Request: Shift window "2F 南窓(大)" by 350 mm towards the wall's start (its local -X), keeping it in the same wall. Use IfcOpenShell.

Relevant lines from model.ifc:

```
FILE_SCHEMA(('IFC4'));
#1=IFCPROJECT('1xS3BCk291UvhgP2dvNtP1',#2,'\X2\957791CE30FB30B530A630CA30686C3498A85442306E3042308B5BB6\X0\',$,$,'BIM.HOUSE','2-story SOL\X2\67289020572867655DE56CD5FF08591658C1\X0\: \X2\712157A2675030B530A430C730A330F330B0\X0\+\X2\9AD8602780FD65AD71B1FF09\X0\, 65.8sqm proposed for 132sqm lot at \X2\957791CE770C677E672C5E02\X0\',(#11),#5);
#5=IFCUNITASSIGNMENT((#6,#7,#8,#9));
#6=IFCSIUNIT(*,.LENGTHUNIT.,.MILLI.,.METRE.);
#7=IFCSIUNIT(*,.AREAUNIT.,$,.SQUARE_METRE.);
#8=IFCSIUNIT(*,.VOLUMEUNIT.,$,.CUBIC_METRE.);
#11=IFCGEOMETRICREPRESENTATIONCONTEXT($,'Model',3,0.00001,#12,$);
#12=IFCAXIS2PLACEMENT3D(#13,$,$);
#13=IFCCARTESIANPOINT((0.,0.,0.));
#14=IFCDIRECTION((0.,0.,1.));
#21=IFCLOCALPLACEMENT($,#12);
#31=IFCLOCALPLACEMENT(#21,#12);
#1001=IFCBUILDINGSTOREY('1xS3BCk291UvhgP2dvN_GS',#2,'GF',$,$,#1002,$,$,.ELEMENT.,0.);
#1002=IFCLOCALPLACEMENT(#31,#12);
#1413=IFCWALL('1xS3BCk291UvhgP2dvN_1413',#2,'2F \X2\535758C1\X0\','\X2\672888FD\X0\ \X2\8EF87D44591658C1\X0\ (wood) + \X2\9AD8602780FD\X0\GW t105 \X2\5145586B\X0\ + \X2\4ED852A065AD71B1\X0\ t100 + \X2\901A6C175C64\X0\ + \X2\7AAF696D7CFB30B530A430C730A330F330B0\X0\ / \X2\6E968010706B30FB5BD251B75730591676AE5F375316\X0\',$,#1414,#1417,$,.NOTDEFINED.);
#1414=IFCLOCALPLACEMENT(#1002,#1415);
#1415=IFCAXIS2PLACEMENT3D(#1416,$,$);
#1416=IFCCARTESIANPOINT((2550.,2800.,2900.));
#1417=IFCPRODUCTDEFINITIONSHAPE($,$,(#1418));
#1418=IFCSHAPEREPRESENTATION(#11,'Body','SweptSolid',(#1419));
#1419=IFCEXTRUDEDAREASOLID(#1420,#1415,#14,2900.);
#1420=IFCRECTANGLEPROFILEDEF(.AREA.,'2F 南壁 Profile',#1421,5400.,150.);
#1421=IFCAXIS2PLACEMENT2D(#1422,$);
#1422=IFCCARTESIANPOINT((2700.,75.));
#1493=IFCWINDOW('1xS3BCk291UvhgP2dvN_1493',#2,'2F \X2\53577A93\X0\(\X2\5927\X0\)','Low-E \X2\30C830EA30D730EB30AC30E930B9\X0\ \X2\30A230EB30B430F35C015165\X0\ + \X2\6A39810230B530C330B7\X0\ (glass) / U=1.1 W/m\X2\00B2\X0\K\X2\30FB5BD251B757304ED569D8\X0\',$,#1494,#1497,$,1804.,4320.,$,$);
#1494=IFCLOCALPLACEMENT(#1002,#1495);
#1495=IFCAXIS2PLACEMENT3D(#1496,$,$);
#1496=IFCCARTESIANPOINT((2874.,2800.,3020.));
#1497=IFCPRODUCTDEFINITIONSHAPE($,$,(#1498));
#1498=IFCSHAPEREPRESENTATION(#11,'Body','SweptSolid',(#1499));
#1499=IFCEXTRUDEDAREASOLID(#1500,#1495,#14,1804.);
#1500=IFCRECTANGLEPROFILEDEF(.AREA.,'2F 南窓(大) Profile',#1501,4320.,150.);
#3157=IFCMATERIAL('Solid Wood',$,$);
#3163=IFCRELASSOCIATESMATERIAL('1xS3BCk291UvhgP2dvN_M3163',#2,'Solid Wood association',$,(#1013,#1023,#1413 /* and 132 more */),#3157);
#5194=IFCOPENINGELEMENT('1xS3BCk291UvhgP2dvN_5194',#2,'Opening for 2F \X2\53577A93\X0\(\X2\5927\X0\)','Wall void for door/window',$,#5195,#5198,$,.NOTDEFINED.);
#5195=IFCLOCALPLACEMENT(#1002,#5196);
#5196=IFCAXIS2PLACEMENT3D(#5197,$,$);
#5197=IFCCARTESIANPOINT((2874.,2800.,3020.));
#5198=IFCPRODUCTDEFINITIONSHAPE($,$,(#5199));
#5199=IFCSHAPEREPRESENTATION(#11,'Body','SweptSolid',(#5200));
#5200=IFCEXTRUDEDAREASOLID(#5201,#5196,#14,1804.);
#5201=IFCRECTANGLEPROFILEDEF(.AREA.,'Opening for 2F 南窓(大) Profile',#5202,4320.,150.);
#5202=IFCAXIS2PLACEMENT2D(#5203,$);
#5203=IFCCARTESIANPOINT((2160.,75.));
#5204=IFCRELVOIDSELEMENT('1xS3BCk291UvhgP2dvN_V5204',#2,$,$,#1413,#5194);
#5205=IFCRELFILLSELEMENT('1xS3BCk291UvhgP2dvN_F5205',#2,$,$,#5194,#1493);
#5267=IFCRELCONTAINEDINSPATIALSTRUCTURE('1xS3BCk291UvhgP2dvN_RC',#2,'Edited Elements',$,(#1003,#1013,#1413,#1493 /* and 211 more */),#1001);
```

```python
import ifcopenshell
import ifcopenshell.api.geometry
import ifcopenshell.util.placement
import ifcopenshell.util.unit

model = ifcopenshell.open("model.ifc")
unit_scale = ifcopenshell.util.unit.calculate_unit_scale(model)

window = model.by_id(1493)
opening = window.FillsVoids[0].RelatingOpeningElement
wall = opening.VoidsElements[0].RelatingBuildingElement

wall_matrix = ifcopenshell.util.placement.get_local_placement(wall.ObjectPlacement)
shift = wall_matrix[:3, 0] * -0.35 / unit_scale
before = ifcopenshell.util.placement.get_local_placement(window.ObjectPlacement)[:3, 3].copy()

# The window is not placed relative to its opening, so move both.
for product in (opening, window):
    matrix = ifcopenshell.util.placement.get_local_placement(product.ObjectPlacement)
    matrix[:3, 3] += shift
    ifcopenshell.api.geometry.edit_object_placement(model, product=product, matrix=matrix, is_si=False)

after = ifcopenshell.util.placement.get_local_placement(window.ObjectPlacement)[:3, 3]
print("window moved by", (after - before).round(3) + 0.0)

model.write("model_rev.ifc")
```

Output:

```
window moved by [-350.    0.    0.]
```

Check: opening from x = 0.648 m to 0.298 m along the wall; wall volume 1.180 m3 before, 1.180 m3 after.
